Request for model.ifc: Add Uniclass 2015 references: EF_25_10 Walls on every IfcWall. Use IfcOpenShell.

First a look at what the model holds.

```python
import ifcopenshell

model = ifcopenshell.open("model.ifc")
print(model.schema)
print("classifications:", [c.Name for c in model.by_type("IfcClassification")])
for ifc_class in ("IfcDoor", "IfcRoof", "IfcStair", "IfcWall", "IfcWindow"):
    print(ifc_class, len(model.by_type(ifc_class)))
```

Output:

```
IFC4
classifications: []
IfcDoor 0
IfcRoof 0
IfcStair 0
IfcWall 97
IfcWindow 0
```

```python
import ifcopenshell
import ifcopenshell.api.classification

model = ifcopenshell.open("model.ifc")

system = ifcopenshell.api.classification.add_classification(model, classification="Uniclass 2015")

codes = {
    "IfcWall": ("EF_25_10", "Walls"),
}
for ifc_class, (code, name) in codes.items():
    products = model.by_type(ifc_class)
    ifcopenshell.api.classification.add_reference(
        model, products=products, classification=system, identification=code, name=name
    )
    print(code, len(products))

model.write("model_v2.ifc")
```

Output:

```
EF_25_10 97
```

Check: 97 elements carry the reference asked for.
